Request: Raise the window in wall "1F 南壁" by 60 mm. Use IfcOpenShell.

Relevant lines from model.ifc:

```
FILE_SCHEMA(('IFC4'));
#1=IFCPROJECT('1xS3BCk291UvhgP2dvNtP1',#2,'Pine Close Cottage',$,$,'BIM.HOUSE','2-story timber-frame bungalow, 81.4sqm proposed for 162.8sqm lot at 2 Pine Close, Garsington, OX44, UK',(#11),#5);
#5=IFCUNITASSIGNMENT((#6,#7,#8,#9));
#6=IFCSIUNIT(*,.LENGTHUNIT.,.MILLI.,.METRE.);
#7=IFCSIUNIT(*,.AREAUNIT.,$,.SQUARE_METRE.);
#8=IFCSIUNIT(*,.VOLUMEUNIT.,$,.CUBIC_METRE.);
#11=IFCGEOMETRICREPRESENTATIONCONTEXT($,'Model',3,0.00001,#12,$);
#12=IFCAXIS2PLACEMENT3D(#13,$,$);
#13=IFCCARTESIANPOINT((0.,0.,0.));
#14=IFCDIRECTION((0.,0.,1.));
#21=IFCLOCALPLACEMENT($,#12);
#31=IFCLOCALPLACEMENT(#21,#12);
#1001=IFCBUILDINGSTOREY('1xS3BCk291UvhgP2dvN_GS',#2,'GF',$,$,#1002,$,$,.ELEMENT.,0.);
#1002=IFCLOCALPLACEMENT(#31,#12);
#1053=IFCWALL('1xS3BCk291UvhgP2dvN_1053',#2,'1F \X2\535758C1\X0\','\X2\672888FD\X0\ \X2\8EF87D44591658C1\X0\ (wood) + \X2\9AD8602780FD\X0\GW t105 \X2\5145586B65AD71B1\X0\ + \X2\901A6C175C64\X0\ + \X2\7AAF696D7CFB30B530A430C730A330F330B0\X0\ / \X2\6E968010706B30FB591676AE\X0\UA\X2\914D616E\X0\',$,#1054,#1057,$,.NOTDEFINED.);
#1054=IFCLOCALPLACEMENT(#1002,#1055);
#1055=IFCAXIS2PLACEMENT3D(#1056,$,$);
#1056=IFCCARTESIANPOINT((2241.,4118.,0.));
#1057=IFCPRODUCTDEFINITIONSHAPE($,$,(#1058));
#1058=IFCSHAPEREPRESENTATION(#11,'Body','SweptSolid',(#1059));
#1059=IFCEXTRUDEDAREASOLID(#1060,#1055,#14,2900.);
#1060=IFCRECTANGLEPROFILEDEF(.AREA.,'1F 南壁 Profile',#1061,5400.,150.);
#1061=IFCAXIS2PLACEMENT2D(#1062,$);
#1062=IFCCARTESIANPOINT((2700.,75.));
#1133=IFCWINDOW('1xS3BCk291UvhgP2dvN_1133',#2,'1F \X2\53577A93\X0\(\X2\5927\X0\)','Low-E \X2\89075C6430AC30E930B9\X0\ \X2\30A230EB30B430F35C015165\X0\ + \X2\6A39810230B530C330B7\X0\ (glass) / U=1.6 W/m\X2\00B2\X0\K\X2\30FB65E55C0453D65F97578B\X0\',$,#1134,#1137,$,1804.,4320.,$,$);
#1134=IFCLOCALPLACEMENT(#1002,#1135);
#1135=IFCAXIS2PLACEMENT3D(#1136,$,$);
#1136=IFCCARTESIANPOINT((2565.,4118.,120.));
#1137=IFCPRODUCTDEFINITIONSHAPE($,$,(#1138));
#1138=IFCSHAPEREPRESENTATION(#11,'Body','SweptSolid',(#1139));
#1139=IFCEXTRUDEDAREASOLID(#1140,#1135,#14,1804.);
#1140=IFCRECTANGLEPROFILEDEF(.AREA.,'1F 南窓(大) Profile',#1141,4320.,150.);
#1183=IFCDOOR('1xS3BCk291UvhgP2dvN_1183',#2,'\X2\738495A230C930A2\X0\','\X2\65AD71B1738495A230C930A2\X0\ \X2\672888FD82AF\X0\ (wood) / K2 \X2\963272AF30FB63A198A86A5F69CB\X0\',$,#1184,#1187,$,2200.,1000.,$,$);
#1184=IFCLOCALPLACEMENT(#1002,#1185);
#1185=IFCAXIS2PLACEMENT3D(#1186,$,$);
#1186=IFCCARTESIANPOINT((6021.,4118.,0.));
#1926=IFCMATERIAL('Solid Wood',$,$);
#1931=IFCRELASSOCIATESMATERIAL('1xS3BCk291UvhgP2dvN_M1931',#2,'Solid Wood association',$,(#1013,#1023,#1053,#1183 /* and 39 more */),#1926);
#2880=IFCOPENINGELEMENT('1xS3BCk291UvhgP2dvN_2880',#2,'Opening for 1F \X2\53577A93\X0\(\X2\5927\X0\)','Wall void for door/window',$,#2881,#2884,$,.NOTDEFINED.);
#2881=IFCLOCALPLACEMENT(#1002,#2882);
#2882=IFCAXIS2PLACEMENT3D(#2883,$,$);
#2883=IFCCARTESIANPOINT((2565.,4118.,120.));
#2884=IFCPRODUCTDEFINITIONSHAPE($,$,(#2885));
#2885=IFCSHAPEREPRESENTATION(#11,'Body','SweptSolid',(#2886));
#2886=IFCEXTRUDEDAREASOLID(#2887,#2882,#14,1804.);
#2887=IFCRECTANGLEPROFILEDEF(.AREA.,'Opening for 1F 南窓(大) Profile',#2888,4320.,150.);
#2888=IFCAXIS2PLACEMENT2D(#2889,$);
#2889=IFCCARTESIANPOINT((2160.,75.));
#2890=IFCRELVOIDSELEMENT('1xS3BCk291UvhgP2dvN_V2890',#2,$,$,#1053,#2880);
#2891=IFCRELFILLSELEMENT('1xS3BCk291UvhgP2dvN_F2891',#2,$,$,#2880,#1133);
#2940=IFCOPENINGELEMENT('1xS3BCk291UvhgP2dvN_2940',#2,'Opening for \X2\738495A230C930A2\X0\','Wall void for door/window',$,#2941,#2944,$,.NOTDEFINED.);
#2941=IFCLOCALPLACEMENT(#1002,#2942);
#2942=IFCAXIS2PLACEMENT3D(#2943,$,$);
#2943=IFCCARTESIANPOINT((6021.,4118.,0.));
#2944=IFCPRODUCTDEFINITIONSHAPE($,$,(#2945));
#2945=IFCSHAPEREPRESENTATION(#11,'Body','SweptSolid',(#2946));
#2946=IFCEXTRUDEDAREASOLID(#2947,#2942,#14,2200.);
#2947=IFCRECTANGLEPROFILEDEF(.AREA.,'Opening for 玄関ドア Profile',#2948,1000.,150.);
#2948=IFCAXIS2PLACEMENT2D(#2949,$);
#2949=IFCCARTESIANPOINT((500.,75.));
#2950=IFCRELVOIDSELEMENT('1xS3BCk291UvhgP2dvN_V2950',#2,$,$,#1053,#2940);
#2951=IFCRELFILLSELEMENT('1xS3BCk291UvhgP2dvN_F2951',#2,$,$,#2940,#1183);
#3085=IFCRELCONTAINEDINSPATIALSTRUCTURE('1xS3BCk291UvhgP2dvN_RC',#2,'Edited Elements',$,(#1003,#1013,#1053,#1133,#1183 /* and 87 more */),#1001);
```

```python
import numpy as np
import ifcopenshell
import ifcopenshell.api.geometry
import ifcopenshell.util.placement
import ifcopenshell.util.unit

model = ifcopenshell.open("model.ifc")
unit_scale = ifcopenshell.util.unit.calculate_unit_scale(model)

window = model.by_guid("1xS3BCk291UvhgP2dvN_1133")
opening = window.FillsVoids[0].RelatingOpeningElement
dz = 0.06 / unit_scale

shift = np.array([0.0, 0.0, dz])
# The window is not placed relative to its opening, so move both.
for product in (opening, window):
    matrix = ifcopenshell.util.placement.get_local_placement(product.ObjectPlacement)
    matrix[:3, 3] += shift
    ifcopenshell.api.geometry.edit_object_placement(model, product=product, matrix=matrix, is_si=False)

print(f"moved by {dz * unit_scale:+.3f} m")

model.write("model_updated.ifc")
```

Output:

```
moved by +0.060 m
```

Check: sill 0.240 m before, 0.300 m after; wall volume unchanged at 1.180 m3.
